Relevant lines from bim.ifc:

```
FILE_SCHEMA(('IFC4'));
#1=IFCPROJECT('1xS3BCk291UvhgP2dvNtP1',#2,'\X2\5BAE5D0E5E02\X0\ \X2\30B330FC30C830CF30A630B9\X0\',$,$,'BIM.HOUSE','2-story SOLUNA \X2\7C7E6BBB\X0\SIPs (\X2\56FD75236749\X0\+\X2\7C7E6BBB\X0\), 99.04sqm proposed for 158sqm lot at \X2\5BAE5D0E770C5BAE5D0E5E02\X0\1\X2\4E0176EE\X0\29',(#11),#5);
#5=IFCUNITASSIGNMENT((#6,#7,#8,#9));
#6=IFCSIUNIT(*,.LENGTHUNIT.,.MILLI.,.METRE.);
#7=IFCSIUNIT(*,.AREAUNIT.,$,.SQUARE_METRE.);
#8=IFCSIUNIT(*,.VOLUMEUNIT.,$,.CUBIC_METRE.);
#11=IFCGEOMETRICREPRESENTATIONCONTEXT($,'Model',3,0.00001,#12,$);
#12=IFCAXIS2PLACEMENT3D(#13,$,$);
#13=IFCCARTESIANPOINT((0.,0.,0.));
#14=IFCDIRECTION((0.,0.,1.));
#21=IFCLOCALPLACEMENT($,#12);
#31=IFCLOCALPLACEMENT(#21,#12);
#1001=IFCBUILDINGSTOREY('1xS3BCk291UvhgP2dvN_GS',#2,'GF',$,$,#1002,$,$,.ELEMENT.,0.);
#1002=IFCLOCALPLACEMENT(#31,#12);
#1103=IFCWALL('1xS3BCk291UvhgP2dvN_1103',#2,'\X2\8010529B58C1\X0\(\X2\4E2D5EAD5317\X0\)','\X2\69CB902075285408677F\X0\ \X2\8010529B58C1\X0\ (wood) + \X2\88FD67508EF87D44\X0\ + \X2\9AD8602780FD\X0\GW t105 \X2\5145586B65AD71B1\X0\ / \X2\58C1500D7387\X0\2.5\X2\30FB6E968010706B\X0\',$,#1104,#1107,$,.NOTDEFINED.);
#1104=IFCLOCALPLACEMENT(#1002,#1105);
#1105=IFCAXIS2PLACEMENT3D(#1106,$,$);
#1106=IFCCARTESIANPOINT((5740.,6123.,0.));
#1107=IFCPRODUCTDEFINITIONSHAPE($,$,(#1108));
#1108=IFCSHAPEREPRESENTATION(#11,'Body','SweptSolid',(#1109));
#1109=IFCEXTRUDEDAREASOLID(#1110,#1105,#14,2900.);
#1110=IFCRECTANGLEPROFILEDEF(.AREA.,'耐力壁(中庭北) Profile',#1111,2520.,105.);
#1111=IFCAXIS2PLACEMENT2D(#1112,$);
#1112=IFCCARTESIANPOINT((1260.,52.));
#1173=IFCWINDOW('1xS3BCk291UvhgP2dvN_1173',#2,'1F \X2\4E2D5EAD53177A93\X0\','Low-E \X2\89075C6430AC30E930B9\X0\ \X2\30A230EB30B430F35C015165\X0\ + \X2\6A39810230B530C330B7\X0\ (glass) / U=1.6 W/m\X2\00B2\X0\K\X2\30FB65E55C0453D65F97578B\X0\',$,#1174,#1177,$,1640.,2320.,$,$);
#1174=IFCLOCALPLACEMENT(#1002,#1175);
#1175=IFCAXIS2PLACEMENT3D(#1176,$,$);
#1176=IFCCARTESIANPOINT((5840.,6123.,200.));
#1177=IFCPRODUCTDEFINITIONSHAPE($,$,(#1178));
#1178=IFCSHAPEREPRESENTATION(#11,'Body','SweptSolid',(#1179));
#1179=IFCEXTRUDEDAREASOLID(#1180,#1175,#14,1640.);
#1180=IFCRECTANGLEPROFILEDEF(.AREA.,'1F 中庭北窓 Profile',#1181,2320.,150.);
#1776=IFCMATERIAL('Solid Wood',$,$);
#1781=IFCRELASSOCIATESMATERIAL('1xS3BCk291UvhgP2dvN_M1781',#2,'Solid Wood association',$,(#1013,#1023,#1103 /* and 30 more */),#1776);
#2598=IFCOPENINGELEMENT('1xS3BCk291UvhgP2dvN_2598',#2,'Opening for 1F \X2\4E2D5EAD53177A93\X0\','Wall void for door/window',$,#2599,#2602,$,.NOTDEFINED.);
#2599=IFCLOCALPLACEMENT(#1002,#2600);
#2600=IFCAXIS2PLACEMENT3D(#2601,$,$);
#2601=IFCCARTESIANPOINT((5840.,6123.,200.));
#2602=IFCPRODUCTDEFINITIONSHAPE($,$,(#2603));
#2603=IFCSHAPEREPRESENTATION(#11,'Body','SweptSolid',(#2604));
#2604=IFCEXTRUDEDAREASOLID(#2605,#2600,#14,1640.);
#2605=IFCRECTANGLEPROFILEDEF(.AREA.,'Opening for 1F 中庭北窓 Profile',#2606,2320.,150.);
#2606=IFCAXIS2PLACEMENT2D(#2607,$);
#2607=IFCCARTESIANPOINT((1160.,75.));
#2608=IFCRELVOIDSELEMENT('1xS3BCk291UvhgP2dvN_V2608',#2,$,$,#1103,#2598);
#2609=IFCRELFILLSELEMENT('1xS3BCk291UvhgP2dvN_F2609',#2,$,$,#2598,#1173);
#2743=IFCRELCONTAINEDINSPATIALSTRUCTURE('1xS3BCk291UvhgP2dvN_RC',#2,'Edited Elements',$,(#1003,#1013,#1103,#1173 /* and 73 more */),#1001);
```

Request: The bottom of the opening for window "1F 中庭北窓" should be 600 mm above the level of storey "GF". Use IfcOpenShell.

```python
import numpy as np
import ifcopenshell
import ifcopenshell.api.geometry
import ifcopenshell.geom
import ifcopenshell.util.element
import ifcopenshell.util.placement
import ifcopenshell.util.shape
import ifcopenshell.util.unit

model = ifcopenshell.open("bim.ifc")
unit_scale = ifcopenshell.util.unit.calculate_unit_scale(model)

window = model.by_id(1173)
opening = window.FillsVoids[0].RelatingOpeningElement
storey = ifcopenshell.util.element.get_container(window, ifc_class="IfcBuildingStorey")
level = ifcopenshell.util.placement.get_local_placement(storey.ObjectPlacement)[2, 3]

# The opening's origin need not be at the sill, so measure its lowest point.
shape = ifcopenshell.geom.create_shape(ifcopenshell.geom.settings(), opening)
bottom = ifcopenshell.util.shape.get_shape_bottom_elevation(shape, shape.geometry) / unit_scale
dz = level + 600.0 - bottom

shift = np.array([0.0, 0.0, dz])
# The window is not placed relative to its opening, so move both.
for product in (opening, window):
    matrix = ifcopenshell.util.placement.get_local_placement(product.ObjectPlacement)
    matrix[:3, 3] += shift
    ifcopenshell.api.geometry.edit_object_placement(model, product=product, matrix=matrix, is_si=False)

print(f"moved by {dz * unit_scale:+.3f} m")

model.write("bim_rev.ifc")
```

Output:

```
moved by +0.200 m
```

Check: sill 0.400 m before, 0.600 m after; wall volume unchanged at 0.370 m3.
